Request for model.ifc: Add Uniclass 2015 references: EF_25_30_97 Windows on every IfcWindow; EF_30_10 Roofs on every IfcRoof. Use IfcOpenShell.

First a look at what the model holds.

```python
import ifcopenshell

model = ifcopenshell.open("model.ifc")
print(model.schema)
print("classifications:", [c.Name for c in model.by_type("IfcClassification")])
for ifc_class in ("IfcDoor", "IfcRoof", "IfcStair", "IfcWall", "IfcWindow"):
    print(ifc_class, len(model.by_type(ifc_class)))
```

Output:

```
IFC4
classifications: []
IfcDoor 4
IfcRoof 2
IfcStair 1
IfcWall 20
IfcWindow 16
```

```python
import ifcopenshell
import ifcopenshell.api.classification

model = ifcopenshell.open("model.ifc")

system = ifcopenshell.api.classification.add_classification(model, classification="Uniclass 2015")

codes = {
    "IfcWindow": ("EF_25_30_97", "Windows"),
    "IfcRoof": ("EF_30_10", "Roofs"),
}
for ifc_class, (code, name) in codes.items():
    products = model.by_type(ifc_class)
    ifcopenshell.api.classification.add_reference(
        model, products=products, classification=system, identification=code, name=name
    )
    print(code, len(products))

model.write("model-out.ifc")
```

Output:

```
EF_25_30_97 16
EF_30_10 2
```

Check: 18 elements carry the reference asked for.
